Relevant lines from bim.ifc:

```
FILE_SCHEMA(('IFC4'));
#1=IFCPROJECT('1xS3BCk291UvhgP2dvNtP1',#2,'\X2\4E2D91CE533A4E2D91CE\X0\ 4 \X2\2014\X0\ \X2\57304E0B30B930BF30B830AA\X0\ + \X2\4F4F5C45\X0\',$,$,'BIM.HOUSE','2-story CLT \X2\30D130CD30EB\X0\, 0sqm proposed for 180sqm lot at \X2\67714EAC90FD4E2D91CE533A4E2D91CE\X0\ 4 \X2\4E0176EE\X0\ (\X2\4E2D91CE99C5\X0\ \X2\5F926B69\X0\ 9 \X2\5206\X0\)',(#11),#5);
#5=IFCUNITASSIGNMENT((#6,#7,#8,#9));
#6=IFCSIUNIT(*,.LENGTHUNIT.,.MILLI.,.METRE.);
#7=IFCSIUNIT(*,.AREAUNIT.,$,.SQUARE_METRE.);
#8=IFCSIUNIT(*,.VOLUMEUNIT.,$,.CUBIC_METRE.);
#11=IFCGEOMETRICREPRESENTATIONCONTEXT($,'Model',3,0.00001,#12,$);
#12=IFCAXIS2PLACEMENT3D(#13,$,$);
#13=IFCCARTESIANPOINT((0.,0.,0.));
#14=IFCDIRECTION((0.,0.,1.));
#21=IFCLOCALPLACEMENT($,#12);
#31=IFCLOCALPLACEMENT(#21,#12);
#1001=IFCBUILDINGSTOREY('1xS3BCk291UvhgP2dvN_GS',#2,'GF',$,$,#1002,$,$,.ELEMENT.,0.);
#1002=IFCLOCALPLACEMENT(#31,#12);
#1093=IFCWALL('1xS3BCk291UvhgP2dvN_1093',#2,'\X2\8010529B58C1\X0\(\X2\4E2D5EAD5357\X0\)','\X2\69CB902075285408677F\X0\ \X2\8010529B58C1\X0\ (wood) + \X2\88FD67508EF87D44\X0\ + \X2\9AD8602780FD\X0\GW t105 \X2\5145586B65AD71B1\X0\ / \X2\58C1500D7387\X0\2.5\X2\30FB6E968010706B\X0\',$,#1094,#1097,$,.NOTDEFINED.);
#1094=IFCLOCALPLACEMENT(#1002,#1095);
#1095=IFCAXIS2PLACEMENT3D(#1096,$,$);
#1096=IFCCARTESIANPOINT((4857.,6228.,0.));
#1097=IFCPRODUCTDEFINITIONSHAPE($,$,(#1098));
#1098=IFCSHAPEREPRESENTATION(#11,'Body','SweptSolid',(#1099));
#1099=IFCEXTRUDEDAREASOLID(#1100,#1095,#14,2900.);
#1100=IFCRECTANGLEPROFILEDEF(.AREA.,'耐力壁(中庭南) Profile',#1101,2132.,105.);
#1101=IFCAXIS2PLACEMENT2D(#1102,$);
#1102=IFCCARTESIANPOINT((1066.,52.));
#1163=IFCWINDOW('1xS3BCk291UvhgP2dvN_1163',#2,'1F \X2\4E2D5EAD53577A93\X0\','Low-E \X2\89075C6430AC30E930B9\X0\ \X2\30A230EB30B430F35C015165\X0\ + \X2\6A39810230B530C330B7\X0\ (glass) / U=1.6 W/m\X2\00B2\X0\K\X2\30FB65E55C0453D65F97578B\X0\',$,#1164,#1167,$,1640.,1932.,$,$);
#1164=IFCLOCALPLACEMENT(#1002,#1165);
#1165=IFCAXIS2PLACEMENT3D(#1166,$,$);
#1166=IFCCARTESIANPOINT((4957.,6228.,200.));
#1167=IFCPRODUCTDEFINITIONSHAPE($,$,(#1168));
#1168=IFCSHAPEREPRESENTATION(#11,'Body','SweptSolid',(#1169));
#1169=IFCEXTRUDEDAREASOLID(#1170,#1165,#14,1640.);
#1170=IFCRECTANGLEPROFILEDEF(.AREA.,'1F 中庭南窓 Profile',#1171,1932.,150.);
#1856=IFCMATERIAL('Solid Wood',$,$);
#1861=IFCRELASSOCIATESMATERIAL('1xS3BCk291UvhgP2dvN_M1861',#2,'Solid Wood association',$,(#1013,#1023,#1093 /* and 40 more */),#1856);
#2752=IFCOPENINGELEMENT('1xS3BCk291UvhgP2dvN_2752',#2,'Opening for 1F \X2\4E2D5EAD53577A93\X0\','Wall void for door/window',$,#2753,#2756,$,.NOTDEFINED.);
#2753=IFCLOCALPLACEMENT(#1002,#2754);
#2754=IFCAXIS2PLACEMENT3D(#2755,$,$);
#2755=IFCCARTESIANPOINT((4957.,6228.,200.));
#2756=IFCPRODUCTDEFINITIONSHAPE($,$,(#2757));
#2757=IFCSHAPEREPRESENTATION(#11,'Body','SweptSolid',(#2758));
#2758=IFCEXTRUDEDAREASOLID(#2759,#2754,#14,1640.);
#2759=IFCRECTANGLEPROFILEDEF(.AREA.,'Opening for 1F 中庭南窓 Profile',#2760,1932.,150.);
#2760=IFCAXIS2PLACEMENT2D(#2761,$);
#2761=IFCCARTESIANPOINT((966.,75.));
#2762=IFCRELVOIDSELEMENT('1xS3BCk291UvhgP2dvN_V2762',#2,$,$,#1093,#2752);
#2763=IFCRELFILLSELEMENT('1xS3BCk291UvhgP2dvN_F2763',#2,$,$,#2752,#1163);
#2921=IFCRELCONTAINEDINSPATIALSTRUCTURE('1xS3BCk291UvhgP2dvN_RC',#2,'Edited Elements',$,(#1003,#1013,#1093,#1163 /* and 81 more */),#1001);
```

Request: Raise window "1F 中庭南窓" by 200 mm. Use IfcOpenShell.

```python
import numpy as np
import ifcopenshell
import ifcopenshell.api.geometry
import ifcopenshell.util.placement
import ifcopenshell.util.unit

model = ifcopenshell.open("bim.ifc")
unit_scale = ifcopenshell.util.unit.calculate_unit_scale(model)

window = model.by_guid("1xS3BCk291UvhgP2dvN_1163")
opening = window.FillsVoids[0].RelatingOpeningElement
dz = 0.2 / unit_scale

shift = np.array([0.0, 0.0, dz])
# The window is not placed relative to its opening, so move both.
for product in (opening, window):
    matrix = ifcopenshell.util.placement.get_local_placement(product.ObjectPlacement)
    matrix[:3, 3] += shift
    ifcopenshell.api.geometry.edit_object_placement(model, product=product, matrix=matrix, is_si=False)

print(f"moved by {dz * unit_scale:+.3f} m")

model.write("bim_updated.ifc")
```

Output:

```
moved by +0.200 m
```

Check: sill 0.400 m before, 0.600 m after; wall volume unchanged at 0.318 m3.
